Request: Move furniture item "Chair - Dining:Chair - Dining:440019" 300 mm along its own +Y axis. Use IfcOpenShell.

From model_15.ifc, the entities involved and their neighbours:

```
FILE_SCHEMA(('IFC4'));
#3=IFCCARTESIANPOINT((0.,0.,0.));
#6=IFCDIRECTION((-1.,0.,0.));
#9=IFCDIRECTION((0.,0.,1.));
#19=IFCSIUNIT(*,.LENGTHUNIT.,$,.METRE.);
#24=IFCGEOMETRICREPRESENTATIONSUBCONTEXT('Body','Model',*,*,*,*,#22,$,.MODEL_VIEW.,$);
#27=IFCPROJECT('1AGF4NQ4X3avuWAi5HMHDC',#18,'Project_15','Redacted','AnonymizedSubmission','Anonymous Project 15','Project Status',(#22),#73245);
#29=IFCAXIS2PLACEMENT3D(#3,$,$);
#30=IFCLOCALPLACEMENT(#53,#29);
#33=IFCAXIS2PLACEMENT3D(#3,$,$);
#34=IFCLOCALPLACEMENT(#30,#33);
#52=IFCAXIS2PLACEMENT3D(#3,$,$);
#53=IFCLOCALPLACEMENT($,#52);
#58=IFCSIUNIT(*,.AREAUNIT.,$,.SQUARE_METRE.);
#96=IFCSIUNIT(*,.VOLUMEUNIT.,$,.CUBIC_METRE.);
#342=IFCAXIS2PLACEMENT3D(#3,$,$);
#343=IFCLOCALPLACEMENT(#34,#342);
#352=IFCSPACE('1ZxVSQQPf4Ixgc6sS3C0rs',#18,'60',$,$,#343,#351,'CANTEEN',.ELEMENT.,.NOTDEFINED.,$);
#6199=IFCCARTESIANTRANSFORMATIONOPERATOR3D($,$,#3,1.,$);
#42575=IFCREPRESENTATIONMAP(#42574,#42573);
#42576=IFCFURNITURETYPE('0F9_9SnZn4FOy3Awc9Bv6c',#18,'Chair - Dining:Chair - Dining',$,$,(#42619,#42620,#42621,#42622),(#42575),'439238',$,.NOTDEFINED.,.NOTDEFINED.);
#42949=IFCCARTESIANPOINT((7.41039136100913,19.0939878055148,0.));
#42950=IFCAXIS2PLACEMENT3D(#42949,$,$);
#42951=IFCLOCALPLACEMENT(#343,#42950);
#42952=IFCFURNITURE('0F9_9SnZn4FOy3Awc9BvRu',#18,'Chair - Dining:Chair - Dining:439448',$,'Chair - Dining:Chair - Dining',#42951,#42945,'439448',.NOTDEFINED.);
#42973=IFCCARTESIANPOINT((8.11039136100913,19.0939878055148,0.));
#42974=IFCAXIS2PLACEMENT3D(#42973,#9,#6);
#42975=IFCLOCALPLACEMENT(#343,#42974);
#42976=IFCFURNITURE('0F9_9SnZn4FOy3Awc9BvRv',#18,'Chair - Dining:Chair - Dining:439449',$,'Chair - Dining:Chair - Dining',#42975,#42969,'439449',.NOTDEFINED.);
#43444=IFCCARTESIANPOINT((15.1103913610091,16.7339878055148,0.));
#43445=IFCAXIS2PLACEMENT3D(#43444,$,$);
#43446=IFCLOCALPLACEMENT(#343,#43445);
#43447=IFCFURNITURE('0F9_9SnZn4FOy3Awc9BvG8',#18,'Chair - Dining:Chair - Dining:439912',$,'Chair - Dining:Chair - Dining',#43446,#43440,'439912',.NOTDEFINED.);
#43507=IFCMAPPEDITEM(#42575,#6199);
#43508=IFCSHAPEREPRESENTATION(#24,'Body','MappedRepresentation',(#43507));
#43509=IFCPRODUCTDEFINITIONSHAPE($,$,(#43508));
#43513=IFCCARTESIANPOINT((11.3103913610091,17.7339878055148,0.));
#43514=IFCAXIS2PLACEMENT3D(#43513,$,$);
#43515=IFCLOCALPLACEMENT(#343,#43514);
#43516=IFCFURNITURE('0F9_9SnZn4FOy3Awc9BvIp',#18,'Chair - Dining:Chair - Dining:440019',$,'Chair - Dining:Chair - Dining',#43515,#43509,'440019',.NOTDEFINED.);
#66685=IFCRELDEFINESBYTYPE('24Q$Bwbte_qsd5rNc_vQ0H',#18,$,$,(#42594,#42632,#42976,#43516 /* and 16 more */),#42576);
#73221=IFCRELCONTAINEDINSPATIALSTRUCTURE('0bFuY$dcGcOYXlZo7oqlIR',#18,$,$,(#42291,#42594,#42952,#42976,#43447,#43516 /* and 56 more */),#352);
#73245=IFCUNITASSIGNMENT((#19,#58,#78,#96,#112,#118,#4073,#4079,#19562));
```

```python
import ifcopenshell
import ifcopenshell.api.geometry
import ifcopenshell.util.placement
import ifcopenshell.util.unit

model = ifcopenshell.open("model_15.ifc")
unit_scale = ifcopenshell.util.unit.calculate_unit_scale(model)

item = model.by_guid("0F9_9SnZn4FOy3Awc9BvIp")
matrix = ifcopenshell.util.placement.get_local_placement(item.ObjectPlacement)
matrix[:3, 3] += matrix[:3, 1] * 0.3 / unit_scale
ifcopenshell.api.geometry.edit_object_placement(model, product=item, matrix=matrix, is_si=False)

print(ifcopenshell.util.placement.get_local_placement(item.ObjectPlacement).round(3) + 0.0)

model.write("model_15_edited.ifc")
```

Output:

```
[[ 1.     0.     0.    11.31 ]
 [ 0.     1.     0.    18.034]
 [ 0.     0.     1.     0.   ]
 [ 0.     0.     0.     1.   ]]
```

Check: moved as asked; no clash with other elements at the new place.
